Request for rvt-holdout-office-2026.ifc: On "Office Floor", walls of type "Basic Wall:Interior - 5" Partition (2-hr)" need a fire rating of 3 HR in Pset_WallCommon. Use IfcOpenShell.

First a look at what the model holds.

```python
import ifcopenshell
import ifcopenshell.util.element

model = ifcopenshell.open("rvt-holdout-office-2026.ifc")
print(model.schema)
storey = next(s for s in model.by_type("IfcBuildingStorey") if s.Name == "Office Floor")
walls = [e for e in ifcopenshell.util.element.get_decomposition(storey) if e.is_a("IfcWall")]
seen = {}
for e in walls:
    element_type = ifcopenshell.util.element.get_type(e)
    key = (element_type.Name if element_type != e and element_type else None, ifcopenshell.util.element.get_pset(e, "Pset_WallCommon", "FireRating"))
    seen[key] = seen.get(key, 0) + 1
for (name, value), count in sorted(seen.items(), key=str):
    print(count, "x", name, "|", value)
```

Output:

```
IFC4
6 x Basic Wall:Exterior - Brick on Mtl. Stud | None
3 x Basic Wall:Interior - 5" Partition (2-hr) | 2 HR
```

```python
import ifcopenshell
import ifcopenshell.api.pset
import ifcopenshell.util.element

model = ifcopenshell.open("rvt-holdout-office-2026.ifc")

storey = next(s for s in model.by_type("IfcBuildingStorey") if s.Name == "Office Floor")
walls = [e for e in ifcopenshell.util.element.get_decomposition(storey) if e.is_a("IfcWall")]

count = 0
for e in walls:
    element_type = ifcopenshell.util.element.get_type(e)
    if element_type in (None, e) or element_type.Name != 'Basic Wall:Interior - 5" Partition (2-hr)':
        continue
    # add_pset returns the element's existing set when there is one.
    pset = ifcopenshell.api.pset.add_pset(model, product=e, name="Pset_WallCommon")
    ifcopenshell.api.pset.edit_pset(model, pset=pset, properties={"FireRating": "3 HR"})
    count += 1

print(count, "walls updated")

model.write("rvt-holdout-office-2026-out.ifc")
```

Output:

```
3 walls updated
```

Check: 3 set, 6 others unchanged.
